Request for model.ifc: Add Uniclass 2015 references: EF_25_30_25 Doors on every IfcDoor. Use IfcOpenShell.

First a look at what the model holds.

```python
import ifcopenshell

model = ifcopenshell.open("model.ifc")
print(model.schema)
print("classifications:", [c.Name for c in model.by_type("IfcClassification")])
for ifc_class in ("IfcDoor", "IfcRoof", "IfcStair", "IfcWall", "IfcWindow"):
    print(ifc_class, len(model.by_type(ifc_class)))
```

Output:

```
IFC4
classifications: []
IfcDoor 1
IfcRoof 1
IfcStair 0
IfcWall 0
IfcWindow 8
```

```python
import ifcopenshell
import ifcopenshell.api.classification

model = ifcopenshell.open("model.ifc")

system = ifcopenshell.api.classification.add_classification(model, classification="Uniclass 2015")

codes = {
    "IfcDoor": ("EF_25_30_25", "Doors"),
}
for ifc_class, (code, name) in codes.items():
    products = model.by_type(ifc_class)
    ifcopenshell.api.classification.add_reference(
        model, products=products, classification=system, identification=code, name=name
    )
    print(code, len(products))

model.write("model_rev.ifc")
```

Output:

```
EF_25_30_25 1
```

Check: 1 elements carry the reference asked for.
